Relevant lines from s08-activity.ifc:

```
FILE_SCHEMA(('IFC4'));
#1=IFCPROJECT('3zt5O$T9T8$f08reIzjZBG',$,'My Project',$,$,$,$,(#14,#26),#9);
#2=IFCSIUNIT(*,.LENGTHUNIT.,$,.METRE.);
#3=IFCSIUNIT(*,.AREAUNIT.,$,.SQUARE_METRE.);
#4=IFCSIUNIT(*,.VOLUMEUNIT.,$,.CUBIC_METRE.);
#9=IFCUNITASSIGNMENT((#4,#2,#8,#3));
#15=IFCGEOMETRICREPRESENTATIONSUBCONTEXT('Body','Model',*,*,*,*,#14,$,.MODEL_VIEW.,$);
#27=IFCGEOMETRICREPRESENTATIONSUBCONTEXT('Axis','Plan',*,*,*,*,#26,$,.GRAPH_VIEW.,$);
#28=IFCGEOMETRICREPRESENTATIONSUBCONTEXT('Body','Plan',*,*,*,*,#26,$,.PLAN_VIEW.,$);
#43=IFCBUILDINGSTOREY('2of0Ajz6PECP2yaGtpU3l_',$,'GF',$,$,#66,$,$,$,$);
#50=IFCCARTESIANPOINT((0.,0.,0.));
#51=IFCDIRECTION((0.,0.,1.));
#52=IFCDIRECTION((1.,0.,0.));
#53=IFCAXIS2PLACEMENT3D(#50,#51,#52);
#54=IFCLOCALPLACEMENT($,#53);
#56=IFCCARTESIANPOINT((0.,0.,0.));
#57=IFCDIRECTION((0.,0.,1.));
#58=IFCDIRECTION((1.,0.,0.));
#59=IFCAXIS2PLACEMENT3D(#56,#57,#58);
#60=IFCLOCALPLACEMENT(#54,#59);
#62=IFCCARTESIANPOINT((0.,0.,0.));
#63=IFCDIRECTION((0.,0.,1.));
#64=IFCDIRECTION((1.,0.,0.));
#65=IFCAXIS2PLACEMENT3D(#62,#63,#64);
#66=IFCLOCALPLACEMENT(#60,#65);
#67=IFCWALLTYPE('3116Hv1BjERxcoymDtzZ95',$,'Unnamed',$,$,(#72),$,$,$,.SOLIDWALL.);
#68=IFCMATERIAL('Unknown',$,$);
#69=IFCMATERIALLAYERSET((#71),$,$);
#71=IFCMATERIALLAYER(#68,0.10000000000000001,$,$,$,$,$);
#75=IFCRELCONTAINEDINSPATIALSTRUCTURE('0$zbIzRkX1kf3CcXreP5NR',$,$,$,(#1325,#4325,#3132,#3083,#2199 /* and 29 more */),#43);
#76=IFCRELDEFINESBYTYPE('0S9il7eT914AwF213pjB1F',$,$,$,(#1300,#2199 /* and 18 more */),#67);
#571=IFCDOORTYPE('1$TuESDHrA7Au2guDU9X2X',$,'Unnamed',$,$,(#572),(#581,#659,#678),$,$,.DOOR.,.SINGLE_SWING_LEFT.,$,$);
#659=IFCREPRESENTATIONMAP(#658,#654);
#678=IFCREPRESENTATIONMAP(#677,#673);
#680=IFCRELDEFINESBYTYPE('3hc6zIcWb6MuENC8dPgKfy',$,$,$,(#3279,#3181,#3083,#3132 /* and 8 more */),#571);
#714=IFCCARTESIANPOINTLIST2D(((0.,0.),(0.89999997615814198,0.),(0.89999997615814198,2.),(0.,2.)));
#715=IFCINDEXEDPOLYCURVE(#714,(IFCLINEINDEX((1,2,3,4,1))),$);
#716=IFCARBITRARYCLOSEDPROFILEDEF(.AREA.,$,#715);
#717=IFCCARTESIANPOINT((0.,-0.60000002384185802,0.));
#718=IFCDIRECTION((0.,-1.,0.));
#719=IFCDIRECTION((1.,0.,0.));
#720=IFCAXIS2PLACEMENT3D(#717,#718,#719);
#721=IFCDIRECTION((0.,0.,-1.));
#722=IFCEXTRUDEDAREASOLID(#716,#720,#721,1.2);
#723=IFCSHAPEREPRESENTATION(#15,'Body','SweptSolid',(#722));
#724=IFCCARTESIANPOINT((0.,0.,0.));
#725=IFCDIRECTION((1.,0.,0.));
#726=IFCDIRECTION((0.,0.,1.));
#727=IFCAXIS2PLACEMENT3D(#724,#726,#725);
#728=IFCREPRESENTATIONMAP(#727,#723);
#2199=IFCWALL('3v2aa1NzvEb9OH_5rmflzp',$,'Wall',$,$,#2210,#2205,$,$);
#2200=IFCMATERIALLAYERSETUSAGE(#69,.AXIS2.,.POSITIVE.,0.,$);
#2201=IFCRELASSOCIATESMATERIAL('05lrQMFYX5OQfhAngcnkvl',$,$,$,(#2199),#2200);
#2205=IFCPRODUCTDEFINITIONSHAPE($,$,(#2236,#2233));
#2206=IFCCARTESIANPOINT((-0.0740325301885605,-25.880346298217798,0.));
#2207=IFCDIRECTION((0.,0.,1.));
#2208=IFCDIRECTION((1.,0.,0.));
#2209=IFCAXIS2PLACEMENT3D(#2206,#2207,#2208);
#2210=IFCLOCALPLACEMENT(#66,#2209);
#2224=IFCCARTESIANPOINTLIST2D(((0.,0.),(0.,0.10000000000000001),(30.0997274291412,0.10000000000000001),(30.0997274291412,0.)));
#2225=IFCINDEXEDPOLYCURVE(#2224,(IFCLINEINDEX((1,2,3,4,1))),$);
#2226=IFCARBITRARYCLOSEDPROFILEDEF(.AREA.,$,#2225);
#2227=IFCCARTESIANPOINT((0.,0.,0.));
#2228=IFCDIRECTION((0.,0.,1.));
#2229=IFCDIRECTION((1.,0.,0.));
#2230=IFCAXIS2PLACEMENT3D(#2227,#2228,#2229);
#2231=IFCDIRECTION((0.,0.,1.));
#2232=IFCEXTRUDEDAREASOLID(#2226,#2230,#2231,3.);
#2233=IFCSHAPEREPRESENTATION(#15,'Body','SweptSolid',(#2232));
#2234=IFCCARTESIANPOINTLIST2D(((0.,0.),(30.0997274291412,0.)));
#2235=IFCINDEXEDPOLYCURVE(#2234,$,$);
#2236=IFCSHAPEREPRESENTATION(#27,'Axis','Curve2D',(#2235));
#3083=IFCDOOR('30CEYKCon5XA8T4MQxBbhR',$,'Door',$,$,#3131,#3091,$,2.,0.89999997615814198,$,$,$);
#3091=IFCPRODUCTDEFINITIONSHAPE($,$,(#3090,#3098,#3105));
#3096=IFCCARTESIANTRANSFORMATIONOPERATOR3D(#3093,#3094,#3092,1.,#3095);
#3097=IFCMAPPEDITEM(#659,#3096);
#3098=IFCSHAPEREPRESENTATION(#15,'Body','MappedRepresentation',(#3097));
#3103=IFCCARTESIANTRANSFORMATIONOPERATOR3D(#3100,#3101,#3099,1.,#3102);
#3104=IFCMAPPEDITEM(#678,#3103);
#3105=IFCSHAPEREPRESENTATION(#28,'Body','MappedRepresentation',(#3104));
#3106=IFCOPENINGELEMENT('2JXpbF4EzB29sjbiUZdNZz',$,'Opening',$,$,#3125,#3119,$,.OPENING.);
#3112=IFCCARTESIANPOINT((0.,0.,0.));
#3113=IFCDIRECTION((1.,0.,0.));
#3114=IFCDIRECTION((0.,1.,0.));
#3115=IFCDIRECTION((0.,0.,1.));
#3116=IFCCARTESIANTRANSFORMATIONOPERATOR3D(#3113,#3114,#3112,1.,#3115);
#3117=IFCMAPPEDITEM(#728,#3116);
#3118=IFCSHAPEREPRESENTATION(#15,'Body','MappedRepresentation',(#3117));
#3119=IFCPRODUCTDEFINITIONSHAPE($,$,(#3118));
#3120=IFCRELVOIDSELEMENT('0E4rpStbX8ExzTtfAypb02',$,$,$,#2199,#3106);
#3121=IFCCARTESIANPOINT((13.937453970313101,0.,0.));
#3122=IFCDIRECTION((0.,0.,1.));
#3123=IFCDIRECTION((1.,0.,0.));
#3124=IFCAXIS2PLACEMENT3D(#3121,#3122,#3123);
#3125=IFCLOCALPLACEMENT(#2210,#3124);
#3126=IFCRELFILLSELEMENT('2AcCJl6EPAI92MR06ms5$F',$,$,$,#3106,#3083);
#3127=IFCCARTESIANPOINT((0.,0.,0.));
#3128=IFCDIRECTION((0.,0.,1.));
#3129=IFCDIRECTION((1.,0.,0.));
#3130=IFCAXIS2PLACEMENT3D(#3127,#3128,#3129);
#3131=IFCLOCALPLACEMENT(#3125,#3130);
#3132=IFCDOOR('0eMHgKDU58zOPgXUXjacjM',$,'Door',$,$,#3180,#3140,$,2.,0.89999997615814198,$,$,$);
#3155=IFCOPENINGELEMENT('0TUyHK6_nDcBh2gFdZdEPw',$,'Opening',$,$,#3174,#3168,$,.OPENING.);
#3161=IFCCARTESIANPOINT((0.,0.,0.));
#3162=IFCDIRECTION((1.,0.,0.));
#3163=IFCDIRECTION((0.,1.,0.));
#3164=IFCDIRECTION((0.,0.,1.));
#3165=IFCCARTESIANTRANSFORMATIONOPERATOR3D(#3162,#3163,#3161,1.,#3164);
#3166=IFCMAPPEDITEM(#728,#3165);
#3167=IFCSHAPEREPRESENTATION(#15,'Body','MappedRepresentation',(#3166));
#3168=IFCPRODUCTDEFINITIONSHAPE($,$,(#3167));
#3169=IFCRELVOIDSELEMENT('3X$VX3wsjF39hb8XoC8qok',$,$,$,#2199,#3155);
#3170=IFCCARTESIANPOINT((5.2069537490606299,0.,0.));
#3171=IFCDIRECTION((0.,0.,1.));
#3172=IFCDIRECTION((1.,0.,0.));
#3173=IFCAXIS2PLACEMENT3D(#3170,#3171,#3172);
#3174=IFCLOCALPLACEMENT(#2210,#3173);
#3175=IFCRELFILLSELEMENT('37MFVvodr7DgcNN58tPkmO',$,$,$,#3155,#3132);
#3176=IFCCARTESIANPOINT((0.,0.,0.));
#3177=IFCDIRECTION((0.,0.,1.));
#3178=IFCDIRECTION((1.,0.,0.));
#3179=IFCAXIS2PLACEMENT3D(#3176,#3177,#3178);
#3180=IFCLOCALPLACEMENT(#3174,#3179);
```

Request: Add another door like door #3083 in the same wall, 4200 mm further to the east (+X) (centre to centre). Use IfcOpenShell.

```python
import ifcopenshell
import ifcopenshell.api.feature
import ifcopenshell.api.geometry
import ifcopenshell.api.root
import ifcopenshell.geom
import ifcopenshell.util.element
import ifcopenshell.util.placement
import ifcopenshell.util.shape

model = ifcopenshell.open("s08-activity.ifc")
settings = ifcopenshell.geom.settings()


def volume(element):
    """Net volume in cubic metres, openings subtracted."""
    shape = ifcopenshell.geom.create_shape(settings, element)
    return ifcopenshell.util.shape.get_volume(shape.geometry)


door = model.by_guid("30CEYKCon5XA8T4MQxBbhR")
opening = door.FillsVoids[0].RelatingOpeningElement
wall = opening.VoidsElements[0].RelatingBuildingElement
before = volume(wall)
shift = ifcopenshell.util.placement.get_local_placement(wall.ObjectPlacement)[:3, 0] * 4.2

# copy_class copies the void relationship, type, container and properties, but no geometry.
new_opening = ifcopenshell.api.root.copy_class(model, product=opening)
new_opening.Representation = ifcopenshell.util.element.copy_deep(
    model, opening.Representation, exclude=["IfcGeometricRepresentationContext", "IfcRepresentationMap"]
)
new_door = ifcopenshell.api.root.copy_class(model, product=door)
new_door.Representation = ifcopenshell.util.element.copy_deep(
    model, door.Representation, exclude=["IfcGeometricRepresentationContext", "IfcRepresentationMap"]
)
ifcopenshell.api.feature.add_filling(model, opening=new_opening, element=new_door)

for old, new in ((opening, new_opening), (door, new_door)):
    matrix = ifcopenshell.util.placement.get_local_placement(old.ObjectPlacement)
    matrix[:3, 3] += shift
    ifcopenshell.api.geometry.edit_object_placement(model, product=new, matrix=matrix, is_si=False)

after = volume(wall)

print(f"wall volume {before:.3f} -> {after:.3f} m3")

model.write("s08-activity-out.ifc")
```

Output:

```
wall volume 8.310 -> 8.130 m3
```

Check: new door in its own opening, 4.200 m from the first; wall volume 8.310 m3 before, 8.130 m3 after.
